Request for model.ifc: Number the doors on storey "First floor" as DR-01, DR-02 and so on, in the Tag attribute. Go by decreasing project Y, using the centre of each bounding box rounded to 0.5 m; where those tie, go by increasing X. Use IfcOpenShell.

First a look at what the model holds.

```python
import ifcopenshell
import ifcopenshell.util.element
import ifcopenshell.util.placement

model = ifcopenshell.open("model.ifc")
print(model.schema)
storey = next(s for s in model.by_type("IfcBuildingStorey") if s.Name == "First floor")
doors = [e for e in ifcopenshell.util.element.get_decomposition(storey) if e.is_a("IfcDoor")]
for e in sorted(doors, key=lambda e: e.id()):
    origin = ifcopenshell.util.placement.get_local_placement(e.ObjectPlacement)[:3, 3]
    print(e.id(), e.Tag, e.Name, origin.round(2) + 0.0, sep=" | ")
```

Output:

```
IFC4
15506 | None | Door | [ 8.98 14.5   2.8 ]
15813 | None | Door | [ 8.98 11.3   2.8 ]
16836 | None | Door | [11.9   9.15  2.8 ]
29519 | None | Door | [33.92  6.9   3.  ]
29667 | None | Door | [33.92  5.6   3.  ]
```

```python
import ifcopenshell
import ifcopenshell.geom
import ifcopenshell.util.element
import ifcopenshell.util.shape

model = ifcopenshell.open("model.ifc")
settings = ifcopenshell.geom.settings()
settings.set("use-world-coords", True)


def centre(element):
    shape = ifcopenshell.geom.create_shape(settings, element)
    return ifcopenshell.util.shape.get_bbox_centroid(shape.geometry)


storey = next(s for s in model.by_type("IfcBuildingStorey") if s.Name == "First floor")
doors = [e for e in ifcopenshell.util.element.get_decomposition(storey) if e.is_a("IfcDoor")]

# Insertion points can sit at a corner or the storey origin, so sort by the geometry (in metres).
centres = {e: centre(e) for e in doors}
doors.sort(key=lambda e: (-round(centres[e][1] / 0.5), centres[e][0]))

for i, e in enumerate(doors, start=1):
    number = f"DR-{i:02d}"
    e.Tag = number
    print(e.id(), number)

model.write("model_v2.ifc")
```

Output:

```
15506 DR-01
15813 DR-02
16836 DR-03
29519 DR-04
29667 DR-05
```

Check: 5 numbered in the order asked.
